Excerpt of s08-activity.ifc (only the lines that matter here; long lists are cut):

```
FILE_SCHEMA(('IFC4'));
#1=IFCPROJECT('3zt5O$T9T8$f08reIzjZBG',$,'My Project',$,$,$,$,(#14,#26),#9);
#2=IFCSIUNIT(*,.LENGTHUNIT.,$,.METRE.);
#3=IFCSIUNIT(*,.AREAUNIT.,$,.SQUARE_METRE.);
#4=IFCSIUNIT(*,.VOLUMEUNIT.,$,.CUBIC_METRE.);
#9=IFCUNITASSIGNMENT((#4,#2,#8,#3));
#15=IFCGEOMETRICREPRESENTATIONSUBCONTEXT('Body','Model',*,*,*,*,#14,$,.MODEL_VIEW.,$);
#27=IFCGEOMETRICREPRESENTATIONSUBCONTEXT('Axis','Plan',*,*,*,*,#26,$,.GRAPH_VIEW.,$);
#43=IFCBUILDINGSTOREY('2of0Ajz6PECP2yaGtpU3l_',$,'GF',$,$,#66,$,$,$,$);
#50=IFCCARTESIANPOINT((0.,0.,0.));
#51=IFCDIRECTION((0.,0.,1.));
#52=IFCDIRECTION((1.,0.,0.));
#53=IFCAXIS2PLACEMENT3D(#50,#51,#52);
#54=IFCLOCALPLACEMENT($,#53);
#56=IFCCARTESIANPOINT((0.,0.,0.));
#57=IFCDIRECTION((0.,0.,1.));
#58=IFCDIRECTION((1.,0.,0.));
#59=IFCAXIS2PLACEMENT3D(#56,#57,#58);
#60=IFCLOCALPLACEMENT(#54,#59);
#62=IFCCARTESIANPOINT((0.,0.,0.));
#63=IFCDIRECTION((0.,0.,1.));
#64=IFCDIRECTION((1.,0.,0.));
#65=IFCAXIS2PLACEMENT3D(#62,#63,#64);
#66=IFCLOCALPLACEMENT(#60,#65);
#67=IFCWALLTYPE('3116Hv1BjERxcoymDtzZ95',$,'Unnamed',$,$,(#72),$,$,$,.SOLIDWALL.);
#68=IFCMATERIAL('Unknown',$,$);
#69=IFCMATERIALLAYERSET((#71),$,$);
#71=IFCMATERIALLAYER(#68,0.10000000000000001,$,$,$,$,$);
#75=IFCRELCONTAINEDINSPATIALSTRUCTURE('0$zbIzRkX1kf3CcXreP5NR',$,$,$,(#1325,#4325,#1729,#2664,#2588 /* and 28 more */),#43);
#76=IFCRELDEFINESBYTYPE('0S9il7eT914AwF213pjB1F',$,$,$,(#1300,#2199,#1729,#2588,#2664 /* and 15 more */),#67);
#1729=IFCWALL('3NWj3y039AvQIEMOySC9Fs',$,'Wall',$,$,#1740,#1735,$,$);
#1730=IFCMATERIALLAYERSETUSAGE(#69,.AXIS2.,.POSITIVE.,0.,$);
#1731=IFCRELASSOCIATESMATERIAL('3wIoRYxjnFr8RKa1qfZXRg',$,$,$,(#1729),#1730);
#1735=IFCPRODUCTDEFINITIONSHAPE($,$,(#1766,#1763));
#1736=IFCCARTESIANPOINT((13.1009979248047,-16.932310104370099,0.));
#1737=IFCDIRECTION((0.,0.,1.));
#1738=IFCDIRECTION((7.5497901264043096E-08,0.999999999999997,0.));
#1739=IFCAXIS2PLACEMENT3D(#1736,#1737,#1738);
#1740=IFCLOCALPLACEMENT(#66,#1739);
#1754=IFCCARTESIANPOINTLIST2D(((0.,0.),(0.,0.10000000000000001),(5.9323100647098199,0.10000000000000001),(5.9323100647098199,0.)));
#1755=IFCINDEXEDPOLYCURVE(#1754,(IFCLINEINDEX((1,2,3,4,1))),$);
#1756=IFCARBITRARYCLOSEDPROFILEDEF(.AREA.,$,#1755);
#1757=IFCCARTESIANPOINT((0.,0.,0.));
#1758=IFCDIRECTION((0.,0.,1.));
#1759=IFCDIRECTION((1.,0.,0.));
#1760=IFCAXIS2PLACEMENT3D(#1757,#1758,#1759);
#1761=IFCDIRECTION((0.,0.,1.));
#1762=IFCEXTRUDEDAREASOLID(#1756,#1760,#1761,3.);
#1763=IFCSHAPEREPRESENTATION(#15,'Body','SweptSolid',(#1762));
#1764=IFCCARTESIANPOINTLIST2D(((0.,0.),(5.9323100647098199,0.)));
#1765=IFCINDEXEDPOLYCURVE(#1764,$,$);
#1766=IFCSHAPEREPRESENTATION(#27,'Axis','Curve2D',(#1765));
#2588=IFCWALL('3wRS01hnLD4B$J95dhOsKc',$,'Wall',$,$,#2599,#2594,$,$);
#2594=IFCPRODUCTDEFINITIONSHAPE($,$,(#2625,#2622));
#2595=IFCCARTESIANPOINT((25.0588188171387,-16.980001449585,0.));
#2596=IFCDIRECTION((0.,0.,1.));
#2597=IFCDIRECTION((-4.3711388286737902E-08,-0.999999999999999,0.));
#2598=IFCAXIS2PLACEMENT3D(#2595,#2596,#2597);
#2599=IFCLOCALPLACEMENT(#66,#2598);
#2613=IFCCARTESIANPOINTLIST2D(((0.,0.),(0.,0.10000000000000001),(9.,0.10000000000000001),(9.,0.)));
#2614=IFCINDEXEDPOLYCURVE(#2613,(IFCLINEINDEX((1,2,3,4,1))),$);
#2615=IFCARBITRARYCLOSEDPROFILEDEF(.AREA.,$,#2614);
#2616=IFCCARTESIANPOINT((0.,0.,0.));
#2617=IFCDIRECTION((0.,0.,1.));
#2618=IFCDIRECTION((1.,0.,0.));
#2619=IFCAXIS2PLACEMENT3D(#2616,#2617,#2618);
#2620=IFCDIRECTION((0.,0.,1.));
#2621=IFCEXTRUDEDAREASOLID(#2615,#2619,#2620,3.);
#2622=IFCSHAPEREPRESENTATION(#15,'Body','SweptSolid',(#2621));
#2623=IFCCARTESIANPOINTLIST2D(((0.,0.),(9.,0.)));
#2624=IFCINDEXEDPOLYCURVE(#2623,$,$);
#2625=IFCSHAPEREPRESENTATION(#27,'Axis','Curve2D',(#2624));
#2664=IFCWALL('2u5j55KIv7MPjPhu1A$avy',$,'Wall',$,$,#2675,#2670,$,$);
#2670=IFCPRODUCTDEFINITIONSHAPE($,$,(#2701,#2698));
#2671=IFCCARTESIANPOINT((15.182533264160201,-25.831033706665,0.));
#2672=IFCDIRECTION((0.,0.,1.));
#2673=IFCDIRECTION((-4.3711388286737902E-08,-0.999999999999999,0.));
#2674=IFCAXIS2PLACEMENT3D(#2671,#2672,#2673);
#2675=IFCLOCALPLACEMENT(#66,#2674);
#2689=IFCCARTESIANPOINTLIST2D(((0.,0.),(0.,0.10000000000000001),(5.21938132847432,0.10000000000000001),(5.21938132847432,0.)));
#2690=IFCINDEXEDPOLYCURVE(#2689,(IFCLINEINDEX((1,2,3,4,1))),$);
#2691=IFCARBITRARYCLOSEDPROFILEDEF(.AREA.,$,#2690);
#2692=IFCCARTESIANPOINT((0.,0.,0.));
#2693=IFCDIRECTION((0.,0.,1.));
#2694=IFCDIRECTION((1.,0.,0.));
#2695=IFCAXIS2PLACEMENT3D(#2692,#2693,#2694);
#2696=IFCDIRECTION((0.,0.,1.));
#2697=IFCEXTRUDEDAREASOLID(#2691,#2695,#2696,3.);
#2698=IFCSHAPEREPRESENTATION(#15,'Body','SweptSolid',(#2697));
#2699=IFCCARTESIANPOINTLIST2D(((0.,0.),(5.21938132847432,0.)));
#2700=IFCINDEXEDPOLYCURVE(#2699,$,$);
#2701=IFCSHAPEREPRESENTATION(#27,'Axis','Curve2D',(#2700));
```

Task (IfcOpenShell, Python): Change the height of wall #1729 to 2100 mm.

```python
import ifcopenshell
import ifcopenshell.geom
import ifcopenshell.util.representation
import ifcopenshell.util.shape
import ifcopenshell.util.unit

model = ifcopenshell.open("s08-activity.ifc")
unit_scale = ifcopenshell.util.unit.calculate_unit_scale(model)
settings = ifcopenshell.geom.settings()


def volume(element):
    """Net volume in cubic metres, openings subtracted."""
    shape = ifcopenshell.geom.create_shape(settings, element)
    return ifcopenshell.util.shape.get_volume(shape.geometry)


wall = model.by_guid("3NWj3y039AvQIEMOySC9Fs")
before = volume(wall)

body = ifcopenshell.util.representation.get_representation(wall, "Model", "Body")
solid = body.Items[0]
old_height = solid.Depth
solid.Depth = 2.1 / unit_scale
after = volume(wall)

print(f"height {old_height:g} -> {solid.Depth:g}, volume {before:.3f} -> {after:.3f} m3")

model.write("s08-activity_updated.ifc")
```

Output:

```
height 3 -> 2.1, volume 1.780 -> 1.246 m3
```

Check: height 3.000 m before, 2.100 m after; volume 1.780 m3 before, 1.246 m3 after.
